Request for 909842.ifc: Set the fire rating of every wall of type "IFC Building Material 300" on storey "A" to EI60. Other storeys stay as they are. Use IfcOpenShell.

First a look at what the model holds.

```python
import ifcopenshell
import ifcopenshell.util.element

model = ifcopenshell.open("909842.ifc")
print(model.schema)
storey = next(s for s in model.by_type("IfcBuildingStorey") if s.Name == "A")
walls = [e for e in ifcopenshell.util.element.get_decomposition(storey) if e.is_a("IfcWall")]
seen = {}
for e in walls:
    element_type = ifcopenshell.util.element.get_type(e)
    key = (element_type.Name if element_type != e and element_type else None, ifcopenshell.util.element.get_pset(e, "Pset_WallCommon", "FireRating"))
    seen[key] = seen.get(key, 0) + 1
for (name, value), count in sorted(seen.items(), key=str):
    print(count, "x", name, "|", value)
```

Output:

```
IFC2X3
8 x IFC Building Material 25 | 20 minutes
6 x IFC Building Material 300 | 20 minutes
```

```python
import ifcopenshell
import ifcopenshell.api.pset
import ifcopenshell.util.element

model = ifcopenshell.open("909842.ifc")

storey = next(s for s in model.by_type("IfcBuildingStorey") if s.Name == "A")
walls = [e for e in ifcopenshell.util.element.get_decomposition(storey) if e.is_a("IfcWall")]

count = 0
for e in walls:
    element_type = ifcopenshell.util.element.get_type(e)
    if element_type in (None, e) or element_type.Name != "IFC Building Material 300":
        continue
    # add_pset returns the element's existing set when there is one.
    pset = ifcopenshell.api.pset.add_pset(model, product=e, name="Pset_WallCommon")
    ifcopenshell.api.pset.edit_pset(model, pset=pset, properties={"FireRating": "EI60"})
    count += 1

print(count, "walls updated")

model.write("909842_rev.ifc")
```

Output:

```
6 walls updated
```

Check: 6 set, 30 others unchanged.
